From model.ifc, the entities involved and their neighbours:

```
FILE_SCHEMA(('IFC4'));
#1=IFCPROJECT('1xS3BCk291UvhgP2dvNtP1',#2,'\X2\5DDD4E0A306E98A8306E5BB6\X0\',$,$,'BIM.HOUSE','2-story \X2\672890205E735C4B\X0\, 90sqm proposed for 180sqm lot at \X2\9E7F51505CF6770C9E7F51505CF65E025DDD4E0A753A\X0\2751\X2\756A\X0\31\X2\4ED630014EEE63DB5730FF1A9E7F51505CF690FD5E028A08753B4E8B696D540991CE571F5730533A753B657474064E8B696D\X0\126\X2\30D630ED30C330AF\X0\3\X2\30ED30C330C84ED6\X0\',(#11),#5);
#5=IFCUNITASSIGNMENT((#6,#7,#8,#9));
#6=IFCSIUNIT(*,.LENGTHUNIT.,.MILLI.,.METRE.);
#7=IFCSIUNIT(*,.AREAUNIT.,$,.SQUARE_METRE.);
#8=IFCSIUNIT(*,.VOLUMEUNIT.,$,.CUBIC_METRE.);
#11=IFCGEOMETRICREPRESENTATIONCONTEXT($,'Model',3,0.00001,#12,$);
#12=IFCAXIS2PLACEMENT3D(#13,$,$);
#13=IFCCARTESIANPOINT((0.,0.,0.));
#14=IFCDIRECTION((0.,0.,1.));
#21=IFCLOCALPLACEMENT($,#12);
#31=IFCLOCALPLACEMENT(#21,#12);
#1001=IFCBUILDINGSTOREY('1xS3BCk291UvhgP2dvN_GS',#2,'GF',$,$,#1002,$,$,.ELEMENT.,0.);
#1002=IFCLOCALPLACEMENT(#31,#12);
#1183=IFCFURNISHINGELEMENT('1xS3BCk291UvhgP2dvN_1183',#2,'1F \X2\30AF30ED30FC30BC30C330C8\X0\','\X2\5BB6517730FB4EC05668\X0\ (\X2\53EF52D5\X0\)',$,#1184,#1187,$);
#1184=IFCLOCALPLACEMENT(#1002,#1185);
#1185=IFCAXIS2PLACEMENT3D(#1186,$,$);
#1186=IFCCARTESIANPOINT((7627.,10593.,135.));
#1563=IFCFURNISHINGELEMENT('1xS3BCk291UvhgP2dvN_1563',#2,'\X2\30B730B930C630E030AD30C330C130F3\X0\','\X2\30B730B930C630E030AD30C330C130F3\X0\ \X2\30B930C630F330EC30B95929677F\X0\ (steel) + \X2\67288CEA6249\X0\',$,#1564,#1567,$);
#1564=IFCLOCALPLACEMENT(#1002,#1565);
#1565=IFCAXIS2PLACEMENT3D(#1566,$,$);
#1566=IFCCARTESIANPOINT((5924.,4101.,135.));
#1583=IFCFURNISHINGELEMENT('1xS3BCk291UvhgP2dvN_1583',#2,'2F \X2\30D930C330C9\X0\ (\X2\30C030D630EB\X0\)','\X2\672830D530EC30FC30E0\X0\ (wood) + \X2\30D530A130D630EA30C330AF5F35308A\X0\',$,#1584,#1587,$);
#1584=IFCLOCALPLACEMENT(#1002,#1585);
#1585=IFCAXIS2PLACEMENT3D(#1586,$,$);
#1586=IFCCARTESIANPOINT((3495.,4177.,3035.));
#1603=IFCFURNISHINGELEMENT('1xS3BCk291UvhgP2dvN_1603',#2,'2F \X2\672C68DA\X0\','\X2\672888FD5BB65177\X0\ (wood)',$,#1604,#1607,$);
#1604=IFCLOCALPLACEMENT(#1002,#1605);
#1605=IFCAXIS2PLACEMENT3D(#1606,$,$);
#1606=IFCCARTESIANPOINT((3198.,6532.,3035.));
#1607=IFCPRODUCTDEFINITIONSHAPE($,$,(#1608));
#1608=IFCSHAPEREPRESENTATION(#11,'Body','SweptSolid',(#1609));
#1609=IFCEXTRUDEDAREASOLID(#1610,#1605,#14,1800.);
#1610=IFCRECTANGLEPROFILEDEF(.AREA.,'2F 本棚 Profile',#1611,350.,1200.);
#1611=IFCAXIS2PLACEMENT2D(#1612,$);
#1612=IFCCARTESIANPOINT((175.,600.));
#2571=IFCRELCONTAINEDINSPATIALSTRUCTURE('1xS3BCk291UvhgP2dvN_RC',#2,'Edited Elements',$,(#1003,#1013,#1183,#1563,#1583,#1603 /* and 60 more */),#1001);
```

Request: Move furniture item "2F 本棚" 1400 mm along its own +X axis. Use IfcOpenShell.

```python
import ifcopenshell
import ifcopenshell.api.geometry
import ifcopenshell.util.placement

model = ifcopenshell.open("model.ifc")

item = model.by_guid("1xS3BCk291UvhgP2dvN_1603")
matrix = ifcopenshell.util.placement.get_local_placement(item.ObjectPlacement)
matrix[:3, 3] += matrix[:3, 0] * 1400.0
ifcopenshell.api.geometry.edit_object_placement(model, product=item, matrix=matrix, is_si=False)

print(ifcopenshell.util.placement.get_local_placement(item.ObjectPlacement).round(3) + 0.0)

model.write("model_rev.ifc")
```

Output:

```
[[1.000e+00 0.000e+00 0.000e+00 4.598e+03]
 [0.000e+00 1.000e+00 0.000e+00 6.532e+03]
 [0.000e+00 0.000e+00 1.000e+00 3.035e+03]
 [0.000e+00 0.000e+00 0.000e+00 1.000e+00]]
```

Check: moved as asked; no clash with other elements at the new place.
